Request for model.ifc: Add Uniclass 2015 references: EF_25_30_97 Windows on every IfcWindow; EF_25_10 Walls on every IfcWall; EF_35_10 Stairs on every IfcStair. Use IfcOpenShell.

First a look at what the model holds.

```python
import ifcopenshell

model = ifcopenshell.open("model.ifc")
print(model.schema)
print("classifications:", [c.Name for c in model.by_type("IfcClassification")])
for ifc_class in ("IfcDoor", "IfcRoof", "IfcStair", "IfcWall", "IfcWindow"):
    print(ifc_class, len(model.by_type(ifc_class)))
```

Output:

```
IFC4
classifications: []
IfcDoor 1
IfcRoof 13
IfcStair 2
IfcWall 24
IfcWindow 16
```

```python
import ifcopenshell
import ifcopenshell.api.classification

model = ifcopenshell.open("model.ifc")

system = ifcopenshell.api.classification.add_classification(model, classification="Uniclass 2015")

codes = {
    "IfcWindow": ("EF_25_30_97", "Windows"),
    "IfcWall": ("EF_25_10", "Walls"),
    "IfcStair": ("EF_35_10", "Stairs"),
}
for ifc_class, (code, name) in codes.items():
    products = model.by_type(ifc_class)
    ifcopenshell.api.classification.add_reference(
        model, products=products, classification=system, identification=code, name=name
    )
    print(code, len(products))

model.write("model-out.ifc")
```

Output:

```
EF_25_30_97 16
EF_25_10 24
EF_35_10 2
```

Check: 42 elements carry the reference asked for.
